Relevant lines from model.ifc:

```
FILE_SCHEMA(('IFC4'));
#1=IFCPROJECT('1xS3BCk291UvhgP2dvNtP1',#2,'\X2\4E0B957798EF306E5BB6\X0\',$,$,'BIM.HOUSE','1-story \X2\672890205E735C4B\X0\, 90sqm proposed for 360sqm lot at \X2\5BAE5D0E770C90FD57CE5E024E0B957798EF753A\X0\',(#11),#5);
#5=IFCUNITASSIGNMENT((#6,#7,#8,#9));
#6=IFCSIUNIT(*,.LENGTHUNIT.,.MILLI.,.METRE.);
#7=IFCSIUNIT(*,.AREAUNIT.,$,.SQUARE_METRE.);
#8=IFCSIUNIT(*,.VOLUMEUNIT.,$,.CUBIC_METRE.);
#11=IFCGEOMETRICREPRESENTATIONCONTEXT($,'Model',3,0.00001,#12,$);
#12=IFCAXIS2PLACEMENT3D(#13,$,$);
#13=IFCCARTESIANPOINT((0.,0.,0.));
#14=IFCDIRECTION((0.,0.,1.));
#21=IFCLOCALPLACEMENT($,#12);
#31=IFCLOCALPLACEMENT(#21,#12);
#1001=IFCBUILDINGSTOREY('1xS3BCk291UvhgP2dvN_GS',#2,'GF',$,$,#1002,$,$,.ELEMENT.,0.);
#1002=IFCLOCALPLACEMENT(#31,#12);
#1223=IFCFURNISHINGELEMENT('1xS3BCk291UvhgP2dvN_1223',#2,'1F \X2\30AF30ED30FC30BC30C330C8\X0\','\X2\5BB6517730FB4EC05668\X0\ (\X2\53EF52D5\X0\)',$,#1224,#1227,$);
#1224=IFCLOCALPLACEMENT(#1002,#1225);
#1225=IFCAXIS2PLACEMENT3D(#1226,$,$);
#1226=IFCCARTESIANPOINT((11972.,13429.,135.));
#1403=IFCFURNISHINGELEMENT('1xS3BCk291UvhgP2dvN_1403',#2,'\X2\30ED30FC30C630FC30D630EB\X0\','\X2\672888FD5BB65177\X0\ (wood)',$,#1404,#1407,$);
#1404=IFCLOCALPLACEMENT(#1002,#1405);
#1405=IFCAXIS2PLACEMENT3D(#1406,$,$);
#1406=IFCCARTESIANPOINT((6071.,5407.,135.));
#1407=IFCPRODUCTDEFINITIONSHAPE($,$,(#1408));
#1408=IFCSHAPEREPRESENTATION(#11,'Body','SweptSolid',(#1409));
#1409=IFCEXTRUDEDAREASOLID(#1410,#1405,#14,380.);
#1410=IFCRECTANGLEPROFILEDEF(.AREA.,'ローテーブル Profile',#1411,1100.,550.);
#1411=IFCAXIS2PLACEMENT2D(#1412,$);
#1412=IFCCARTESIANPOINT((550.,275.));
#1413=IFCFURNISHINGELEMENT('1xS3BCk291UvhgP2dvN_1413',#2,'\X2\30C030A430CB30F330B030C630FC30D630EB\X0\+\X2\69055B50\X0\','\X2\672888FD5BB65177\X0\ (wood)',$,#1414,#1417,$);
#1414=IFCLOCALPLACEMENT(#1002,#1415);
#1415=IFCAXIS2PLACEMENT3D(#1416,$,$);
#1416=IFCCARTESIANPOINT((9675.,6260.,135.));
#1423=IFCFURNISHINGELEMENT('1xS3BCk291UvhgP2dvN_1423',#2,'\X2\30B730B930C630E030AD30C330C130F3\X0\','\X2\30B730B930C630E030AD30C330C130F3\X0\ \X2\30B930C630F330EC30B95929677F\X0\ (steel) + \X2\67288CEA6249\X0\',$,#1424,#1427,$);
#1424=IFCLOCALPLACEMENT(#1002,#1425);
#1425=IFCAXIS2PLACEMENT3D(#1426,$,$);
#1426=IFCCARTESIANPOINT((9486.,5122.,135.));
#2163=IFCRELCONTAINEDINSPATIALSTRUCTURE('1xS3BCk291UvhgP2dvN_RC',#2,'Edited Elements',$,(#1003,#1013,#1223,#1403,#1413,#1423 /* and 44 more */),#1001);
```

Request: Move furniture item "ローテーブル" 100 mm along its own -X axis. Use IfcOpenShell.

```python
import ifcopenshell
import ifcopenshell.api.geometry
import ifcopenshell.util.placement
import ifcopenshell.util.unit

model = ifcopenshell.open("model.ifc")
unit_scale = ifcopenshell.util.unit.calculate_unit_scale(model)

item = model.by_guid("1xS3BCk291UvhgP2dvN_1403")
matrix = ifcopenshell.util.placement.get_local_placement(item.ObjectPlacement)
matrix[:3, 3] -= matrix[:3, 0] * 0.1 / unit_scale
ifcopenshell.api.geometry.edit_object_placement(model, product=item, matrix=matrix, is_si=False)

print(ifcopenshell.util.placement.get_local_placement(item.ObjectPlacement).round(3) + 0.0)

model.write("model_updated.ifc")
```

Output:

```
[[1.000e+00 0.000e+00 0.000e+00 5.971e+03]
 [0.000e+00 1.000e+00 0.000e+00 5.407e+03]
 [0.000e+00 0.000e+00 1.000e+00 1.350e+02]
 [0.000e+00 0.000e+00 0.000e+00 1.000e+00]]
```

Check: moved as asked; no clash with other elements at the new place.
